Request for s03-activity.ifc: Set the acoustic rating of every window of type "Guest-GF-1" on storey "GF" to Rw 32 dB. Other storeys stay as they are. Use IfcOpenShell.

First a look at what the model holds.

```python
import ifcopenshell
import ifcopenshell.util.element

model = ifcopenshell.open("s03-activity.ifc")
print(model.schema)
storey = next(s for s in model.by_type("IfcBuildingStorey") if s.Name == "GF")
windows = [e for e in ifcopenshell.util.element.get_decomposition(storey) if e.is_a("IfcWindow")]
seen = {}
for e in windows:
    element_type = ifcopenshell.util.element.get_type(e)
    key = (element_type.Name if element_type != e and element_type else None, ifcopenshell.util.element.get_pset(e, "Pset_WindowCommon", "AcousticRating"))
    seen[key] = seen.get(key, 0) + 1
for (name, value), count in sorted(seen.items(), key=str):
    print(count, "x", name, "|", value)
```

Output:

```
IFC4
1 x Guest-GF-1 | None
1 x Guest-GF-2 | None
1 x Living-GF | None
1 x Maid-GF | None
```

```python
import ifcopenshell
import ifcopenshell.api.pset
import ifcopenshell.util.element

model = ifcopenshell.open("s03-activity.ifc")

storey = next(s for s in model.by_type("IfcBuildingStorey") if s.Name == "GF")
windows = [e for e in ifcopenshell.util.element.get_decomposition(storey) if e.is_a("IfcWindow")]

count = 0
for e in windows:
    element_type = ifcopenshell.util.element.get_type(e)
    if element_type in (None, e) or element_type.Name != "Guest-GF-1":
        continue
    # add_pset returns the element's existing set when there is one.
    pset = ifcopenshell.api.pset.add_pset(model, product=e, name="Pset_WindowCommon")
    ifcopenshell.api.pset.edit_pset(model, pset=pset, properties={"AcousticRating": "Rw 32 dB"})
    count += 1

print(count, "windows updated")

model.write("s03-activity_rev.ifc")
```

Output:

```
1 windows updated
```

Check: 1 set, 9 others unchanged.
